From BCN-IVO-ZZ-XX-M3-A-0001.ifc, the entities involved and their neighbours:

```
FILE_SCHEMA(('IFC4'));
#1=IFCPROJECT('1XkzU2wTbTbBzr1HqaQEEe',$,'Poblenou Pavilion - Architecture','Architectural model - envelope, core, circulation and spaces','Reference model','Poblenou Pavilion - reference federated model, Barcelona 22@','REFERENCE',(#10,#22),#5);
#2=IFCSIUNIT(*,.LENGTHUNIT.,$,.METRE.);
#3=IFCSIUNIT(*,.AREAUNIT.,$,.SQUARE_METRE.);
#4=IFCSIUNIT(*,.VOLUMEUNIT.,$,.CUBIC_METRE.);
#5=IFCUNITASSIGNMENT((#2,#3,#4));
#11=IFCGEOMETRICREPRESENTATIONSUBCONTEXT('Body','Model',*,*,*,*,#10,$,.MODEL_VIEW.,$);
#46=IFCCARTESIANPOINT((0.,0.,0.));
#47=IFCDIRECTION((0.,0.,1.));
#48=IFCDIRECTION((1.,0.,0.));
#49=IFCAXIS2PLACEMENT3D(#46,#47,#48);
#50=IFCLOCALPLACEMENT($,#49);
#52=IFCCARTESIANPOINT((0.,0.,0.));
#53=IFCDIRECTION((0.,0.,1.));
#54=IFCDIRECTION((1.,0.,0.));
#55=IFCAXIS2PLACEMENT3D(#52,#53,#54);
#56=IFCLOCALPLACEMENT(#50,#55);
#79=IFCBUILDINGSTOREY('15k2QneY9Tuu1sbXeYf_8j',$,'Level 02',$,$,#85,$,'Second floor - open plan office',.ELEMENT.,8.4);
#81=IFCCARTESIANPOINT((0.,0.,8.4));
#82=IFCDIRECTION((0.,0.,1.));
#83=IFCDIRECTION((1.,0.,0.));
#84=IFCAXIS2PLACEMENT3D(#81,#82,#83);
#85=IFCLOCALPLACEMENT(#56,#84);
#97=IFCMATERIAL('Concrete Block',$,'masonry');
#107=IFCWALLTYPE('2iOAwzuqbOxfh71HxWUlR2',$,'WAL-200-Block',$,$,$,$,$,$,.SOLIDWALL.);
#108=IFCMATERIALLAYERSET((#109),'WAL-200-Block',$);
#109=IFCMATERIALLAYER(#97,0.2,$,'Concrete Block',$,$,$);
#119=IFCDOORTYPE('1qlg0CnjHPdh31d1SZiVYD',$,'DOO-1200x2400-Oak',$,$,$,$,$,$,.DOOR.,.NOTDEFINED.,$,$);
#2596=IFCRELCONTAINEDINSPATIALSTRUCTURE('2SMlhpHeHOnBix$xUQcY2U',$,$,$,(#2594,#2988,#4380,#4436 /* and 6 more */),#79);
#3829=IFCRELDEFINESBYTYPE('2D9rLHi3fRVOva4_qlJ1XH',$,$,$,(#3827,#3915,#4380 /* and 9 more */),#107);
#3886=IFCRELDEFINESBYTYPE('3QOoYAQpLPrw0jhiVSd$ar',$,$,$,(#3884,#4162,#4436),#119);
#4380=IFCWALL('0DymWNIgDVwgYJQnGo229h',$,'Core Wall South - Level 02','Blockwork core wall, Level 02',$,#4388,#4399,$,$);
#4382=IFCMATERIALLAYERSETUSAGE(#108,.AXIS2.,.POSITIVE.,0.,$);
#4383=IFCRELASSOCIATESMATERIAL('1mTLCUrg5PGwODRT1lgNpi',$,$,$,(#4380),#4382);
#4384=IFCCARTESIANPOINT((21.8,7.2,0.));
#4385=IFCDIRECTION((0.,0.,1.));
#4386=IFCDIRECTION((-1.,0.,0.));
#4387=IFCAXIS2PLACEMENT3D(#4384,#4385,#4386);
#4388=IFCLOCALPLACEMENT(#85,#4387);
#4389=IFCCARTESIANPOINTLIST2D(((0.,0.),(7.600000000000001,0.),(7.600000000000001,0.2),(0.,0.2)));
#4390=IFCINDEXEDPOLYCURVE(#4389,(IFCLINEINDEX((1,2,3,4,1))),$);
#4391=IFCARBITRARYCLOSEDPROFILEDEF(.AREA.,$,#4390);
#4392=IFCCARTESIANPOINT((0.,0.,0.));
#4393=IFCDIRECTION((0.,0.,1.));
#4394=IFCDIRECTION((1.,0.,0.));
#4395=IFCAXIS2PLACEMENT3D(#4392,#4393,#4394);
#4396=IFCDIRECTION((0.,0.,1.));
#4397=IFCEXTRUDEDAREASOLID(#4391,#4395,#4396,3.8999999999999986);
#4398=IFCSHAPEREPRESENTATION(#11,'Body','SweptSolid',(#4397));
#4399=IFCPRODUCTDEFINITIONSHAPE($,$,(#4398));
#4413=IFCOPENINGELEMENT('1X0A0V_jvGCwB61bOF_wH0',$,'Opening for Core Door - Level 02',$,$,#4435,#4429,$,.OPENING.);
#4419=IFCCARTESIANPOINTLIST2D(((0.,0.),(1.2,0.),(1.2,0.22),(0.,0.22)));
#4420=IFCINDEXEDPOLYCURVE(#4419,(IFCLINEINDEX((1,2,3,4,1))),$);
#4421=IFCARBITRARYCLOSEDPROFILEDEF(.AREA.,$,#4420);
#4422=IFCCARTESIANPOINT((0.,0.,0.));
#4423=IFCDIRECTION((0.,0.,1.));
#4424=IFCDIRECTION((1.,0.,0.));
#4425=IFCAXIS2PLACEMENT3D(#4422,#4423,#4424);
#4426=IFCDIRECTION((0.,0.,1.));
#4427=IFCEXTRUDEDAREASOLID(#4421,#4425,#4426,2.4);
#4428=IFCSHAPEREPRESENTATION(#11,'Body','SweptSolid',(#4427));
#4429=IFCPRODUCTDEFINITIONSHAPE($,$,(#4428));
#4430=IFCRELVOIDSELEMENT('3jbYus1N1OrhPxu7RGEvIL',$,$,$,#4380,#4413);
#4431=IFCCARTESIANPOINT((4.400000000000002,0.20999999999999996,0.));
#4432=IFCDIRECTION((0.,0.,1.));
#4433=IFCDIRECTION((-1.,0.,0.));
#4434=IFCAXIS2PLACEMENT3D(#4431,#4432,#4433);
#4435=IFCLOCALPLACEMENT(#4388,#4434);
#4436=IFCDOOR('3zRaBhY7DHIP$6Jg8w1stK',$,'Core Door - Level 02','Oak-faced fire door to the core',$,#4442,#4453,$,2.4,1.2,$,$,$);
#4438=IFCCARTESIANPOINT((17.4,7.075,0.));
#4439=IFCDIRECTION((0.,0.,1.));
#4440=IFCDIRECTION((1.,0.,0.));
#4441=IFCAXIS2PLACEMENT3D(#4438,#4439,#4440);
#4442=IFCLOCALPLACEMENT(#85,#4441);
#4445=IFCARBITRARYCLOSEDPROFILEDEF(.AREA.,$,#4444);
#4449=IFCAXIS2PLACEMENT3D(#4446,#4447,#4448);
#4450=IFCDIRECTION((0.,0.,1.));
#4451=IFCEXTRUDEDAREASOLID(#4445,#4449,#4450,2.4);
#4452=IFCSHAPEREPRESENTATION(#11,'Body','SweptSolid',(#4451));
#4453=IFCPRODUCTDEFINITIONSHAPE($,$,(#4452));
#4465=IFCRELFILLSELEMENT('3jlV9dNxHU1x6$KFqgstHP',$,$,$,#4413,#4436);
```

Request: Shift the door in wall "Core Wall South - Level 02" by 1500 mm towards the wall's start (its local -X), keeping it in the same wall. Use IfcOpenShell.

```python
import ifcopenshell
import ifcopenshell.api.geometry
import ifcopenshell.util.placement
import ifcopenshell.util.unit

model = ifcopenshell.open("BCN-IVO-ZZ-XX-M3-A-0001.ifc")
unit_scale = ifcopenshell.util.unit.calculate_unit_scale(model)

door = model.by_id(4436)
opening = door.FillsVoids[0].RelatingOpeningElement
wall = opening.VoidsElements[0].RelatingBuildingElement

wall_matrix = ifcopenshell.util.placement.get_local_placement(wall.ObjectPlacement)
shift = wall_matrix[:3, 0] * -1.5 / unit_scale
before = ifcopenshell.util.placement.get_local_placement(door.ObjectPlacement)[:3, 3].copy()

# The door is not placed relative to its opening, so move both.
for product in (opening, door):
    matrix = ifcopenshell.util.placement.get_local_placement(product.ObjectPlacement)
    matrix[:3, 3] += shift
    ifcopenshell.api.geometry.edit_object_placement(model, product=product, matrix=matrix, is_si=False)

after = ifcopenshell.util.placement.get_local_placement(door.ObjectPlacement)[:3, 3]
print("door moved by", (after - before).round(3) + 0.0)

model.write("BCN-IVO-ZZ-XX-M3-A-0001-out.ifc")
```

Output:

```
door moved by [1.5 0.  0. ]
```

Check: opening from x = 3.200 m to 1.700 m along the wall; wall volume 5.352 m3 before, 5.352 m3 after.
